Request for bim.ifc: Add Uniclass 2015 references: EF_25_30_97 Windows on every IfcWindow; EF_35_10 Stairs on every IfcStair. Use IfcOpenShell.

First a look at what the model holds.

```python
import ifcopenshell

model = ifcopenshell.open("bim.ifc")
print(model.schema)
print("classifications:", [c.Name for c in model.by_type("IfcClassification")])
for ifc_class in ("IfcDoor", "IfcRoof", "IfcStair", "IfcWall", "IfcWindow"):
    print(ifc_class, len(model.by_type(ifc_class)))
```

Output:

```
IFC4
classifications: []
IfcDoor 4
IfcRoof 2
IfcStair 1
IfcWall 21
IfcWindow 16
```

```python
import ifcopenshell
import ifcopenshell.api.classification

model = ifcopenshell.open("bim.ifc")

system = ifcopenshell.api.classification.add_classification(model, classification="Uniclass 2015")

codes = {
    "IfcWindow": ("EF_25_30_97", "Windows"),
    "IfcStair": ("EF_35_10", "Stairs"),
}
for ifc_class, (code, name) in codes.items():
    products = model.by_type(ifc_class)
    ifcopenshell.api.classification.add_reference(
        model, products=products, classification=system, identification=code, name=name
    )
    print(code, len(products))

model.write("bim_updated.ifc")
```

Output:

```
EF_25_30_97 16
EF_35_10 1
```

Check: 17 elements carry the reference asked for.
